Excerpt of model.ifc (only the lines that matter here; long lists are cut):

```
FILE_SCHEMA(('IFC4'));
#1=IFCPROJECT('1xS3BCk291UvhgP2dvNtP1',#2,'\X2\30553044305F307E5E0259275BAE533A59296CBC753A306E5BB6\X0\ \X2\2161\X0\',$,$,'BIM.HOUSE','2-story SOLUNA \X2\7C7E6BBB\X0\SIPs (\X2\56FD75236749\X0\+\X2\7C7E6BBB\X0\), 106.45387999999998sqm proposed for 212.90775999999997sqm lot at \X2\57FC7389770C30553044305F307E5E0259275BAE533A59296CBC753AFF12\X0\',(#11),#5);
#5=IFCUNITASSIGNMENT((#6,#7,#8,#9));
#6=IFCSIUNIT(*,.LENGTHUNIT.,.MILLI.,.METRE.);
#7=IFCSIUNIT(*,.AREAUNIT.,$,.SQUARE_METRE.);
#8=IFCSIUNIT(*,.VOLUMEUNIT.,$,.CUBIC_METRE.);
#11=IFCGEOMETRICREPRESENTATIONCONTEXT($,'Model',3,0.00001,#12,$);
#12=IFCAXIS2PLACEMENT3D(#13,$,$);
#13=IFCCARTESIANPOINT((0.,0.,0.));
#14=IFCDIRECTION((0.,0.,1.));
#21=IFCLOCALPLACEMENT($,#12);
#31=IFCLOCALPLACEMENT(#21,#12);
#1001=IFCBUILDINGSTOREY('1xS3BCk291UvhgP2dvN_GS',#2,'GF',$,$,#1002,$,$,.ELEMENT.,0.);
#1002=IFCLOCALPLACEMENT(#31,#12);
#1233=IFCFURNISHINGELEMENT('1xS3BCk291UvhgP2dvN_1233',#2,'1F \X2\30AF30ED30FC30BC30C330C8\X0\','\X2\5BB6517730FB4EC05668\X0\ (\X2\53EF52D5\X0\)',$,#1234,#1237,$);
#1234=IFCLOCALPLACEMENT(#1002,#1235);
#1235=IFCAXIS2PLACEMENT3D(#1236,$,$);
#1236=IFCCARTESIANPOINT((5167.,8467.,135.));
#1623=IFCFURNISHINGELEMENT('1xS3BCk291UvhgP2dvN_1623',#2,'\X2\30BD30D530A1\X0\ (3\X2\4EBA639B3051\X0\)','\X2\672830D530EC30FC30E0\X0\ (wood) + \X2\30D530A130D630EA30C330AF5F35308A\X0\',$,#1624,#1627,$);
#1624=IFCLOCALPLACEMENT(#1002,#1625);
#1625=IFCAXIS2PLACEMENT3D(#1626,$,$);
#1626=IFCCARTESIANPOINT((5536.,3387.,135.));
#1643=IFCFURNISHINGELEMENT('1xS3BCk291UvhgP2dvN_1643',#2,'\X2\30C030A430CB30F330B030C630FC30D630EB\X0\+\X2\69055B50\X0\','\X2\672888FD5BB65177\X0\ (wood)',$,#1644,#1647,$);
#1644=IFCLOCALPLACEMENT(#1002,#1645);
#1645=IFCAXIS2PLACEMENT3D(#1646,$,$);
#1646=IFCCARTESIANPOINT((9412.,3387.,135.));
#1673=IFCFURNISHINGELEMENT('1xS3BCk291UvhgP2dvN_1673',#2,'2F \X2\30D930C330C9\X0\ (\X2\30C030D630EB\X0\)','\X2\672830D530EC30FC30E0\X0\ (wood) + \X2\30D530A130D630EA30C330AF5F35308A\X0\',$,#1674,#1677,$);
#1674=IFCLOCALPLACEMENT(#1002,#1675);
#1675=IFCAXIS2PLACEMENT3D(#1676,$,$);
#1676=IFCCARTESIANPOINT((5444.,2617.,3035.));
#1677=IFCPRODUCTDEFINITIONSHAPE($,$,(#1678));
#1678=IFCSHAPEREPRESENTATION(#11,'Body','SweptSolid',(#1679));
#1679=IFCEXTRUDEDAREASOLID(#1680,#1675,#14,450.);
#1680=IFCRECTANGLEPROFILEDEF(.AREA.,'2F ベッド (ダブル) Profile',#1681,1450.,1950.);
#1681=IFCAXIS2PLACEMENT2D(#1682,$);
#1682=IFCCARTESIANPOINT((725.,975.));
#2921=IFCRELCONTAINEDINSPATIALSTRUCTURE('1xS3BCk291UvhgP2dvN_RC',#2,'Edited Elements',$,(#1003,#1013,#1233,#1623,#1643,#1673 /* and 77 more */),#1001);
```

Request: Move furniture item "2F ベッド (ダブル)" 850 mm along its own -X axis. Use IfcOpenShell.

```python
import ifcopenshell
import ifcopenshell.api.geometry
import ifcopenshell.util.placement
import ifcopenshell.util.unit

model = ifcopenshell.open("model.ifc")
unit_scale = ifcopenshell.util.unit.calculate_unit_scale(model)

item = model.by_guid("1xS3BCk291UvhgP2dvN_1673")
matrix = ifcopenshell.util.placement.get_local_placement(item.ObjectPlacement)
matrix[:3, 3] -= matrix[:3, 0] * 0.85 / unit_scale
ifcopenshell.api.geometry.edit_object_placement(model, product=item, matrix=matrix, is_si=False)

print(ifcopenshell.util.placement.get_local_placement(item.ObjectPlacement).round(3) + 0.0)

model.write("model_edited.ifc")
```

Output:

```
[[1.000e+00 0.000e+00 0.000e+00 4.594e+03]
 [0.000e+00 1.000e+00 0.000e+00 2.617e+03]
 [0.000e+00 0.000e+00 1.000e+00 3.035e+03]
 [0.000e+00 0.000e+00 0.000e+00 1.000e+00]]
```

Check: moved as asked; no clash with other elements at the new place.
